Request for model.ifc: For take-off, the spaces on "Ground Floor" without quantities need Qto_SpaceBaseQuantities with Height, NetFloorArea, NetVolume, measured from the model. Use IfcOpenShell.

First a look at what the model holds.

```python
import ifcopenshell
import ifcopenshell.util.element
import ifcopenshell.util.unit

model = ifcopenshell.open("model.ifc")
print(model.schema)
for unit_type in ("LENGTHUNIT", "AREAUNIT", "VOLUMEUNIT"):
    print(unit_type, ifcopenshell.util.unit.calculate_unit_scale(model, unit_type))
storey = next(s for s in model.by_type("IfcBuildingStorey") if s.Name == "Ground Floor")
spaces = [e for e in ifcopenshell.util.element.get_decomposition(storey) if e.is_a("IfcSpace")]
for e in sorted(spaces, key=lambda e: e.id()):
    print(e.id(), e.is_a(), e.Name, list(ifcopenshell.util.element.get_psets(e, qtos_only=True)), sep=" | ")
```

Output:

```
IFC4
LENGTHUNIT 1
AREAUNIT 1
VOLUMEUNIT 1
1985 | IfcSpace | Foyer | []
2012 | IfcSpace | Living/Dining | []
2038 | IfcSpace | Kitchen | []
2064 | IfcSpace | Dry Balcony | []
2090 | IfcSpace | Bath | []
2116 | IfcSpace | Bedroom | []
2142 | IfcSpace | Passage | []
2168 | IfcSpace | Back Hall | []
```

```python
import ifcopenshell
import ifcopenshell.api.pset
import ifcopenshell.geom
import ifcopenshell.util.element
import ifcopenshell.util.shape
import ifcopenshell.util.unit

model = ifcopenshell.open("model.ifc")
unit_scale = ifcopenshell.util.unit.calculate_unit_scale(model)
area_scale = ifcopenshell.util.unit.calculate_unit_scale(model, "AREAUNIT")
volume_scale = ifcopenshell.util.unit.calculate_unit_scale(model, "VOLUMEUNIT")
settings = ifcopenshell.geom.settings()

storey = next(s for s in model.by_type("IfcBuildingStorey") if s.Name == "Ground Floor")
spaces = [e for e in ifcopenshell.util.element.get_decomposition(storey) if e.is_a("IfcSpace")]

for e in sorted(spaces, key=lambda e: e.id()):
    if ifcopenshell.util.element.get_psets(e, qtos_only=True, should_inherit=False):
        continue
    # Geometry comes back in metres, in the element's own axes.
    shape = ifcopenshell.geom.create_shape(settings, e)
    values = {
        "Height": ifcopenshell.util.shape.get_z(shape.geometry) / unit_scale,
        "NetFloorArea": ifcopenshell.util.shape.get_footprint_area(shape.geometry) / area_scale,
        "NetVolume": ifcopenshell.util.shape.get_volume(shape.geometry) / volume_scale,
    }
    qto = ifcopenshell.api.pset.add_qto(model, product=e, name="Qto_SpaceBaseQuantities")
    ifcopenshell.api.pset.edit_qto(model, qto=qto, properties=values)
    print(e.id(), {k: round(v, 3) for k, v in values.items()})

model.write("model_v2.ifc")
```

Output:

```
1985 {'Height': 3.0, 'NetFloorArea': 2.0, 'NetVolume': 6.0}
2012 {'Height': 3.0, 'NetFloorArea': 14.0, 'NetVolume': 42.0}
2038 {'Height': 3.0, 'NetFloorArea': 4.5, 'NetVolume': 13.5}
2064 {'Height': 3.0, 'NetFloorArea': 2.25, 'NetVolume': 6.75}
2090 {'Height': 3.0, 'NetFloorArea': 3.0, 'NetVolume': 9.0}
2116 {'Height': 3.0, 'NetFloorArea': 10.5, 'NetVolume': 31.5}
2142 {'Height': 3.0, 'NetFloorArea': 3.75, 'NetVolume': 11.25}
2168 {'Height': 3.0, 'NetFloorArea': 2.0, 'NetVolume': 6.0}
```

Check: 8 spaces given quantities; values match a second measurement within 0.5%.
